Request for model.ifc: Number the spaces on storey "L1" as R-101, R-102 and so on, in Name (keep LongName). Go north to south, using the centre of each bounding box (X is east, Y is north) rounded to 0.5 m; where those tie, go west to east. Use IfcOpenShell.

First a look at what the model holds.

```python
import ifcopenshell
import ifcopenshell.util.element
import ifcopenshell.util.placement

model = ifcopenshell.open("model.ifc")
print(model.schema)
storey = next(s for s in model.by_type("IfcBuildingStorey") if s.Name == "L1")
spaces = [e for e in ifcopenshell.util.element.get_decomposition(storey) if e.is_a("IfcSpace")]
for e in sorted(spaces, key=lambda e: e.id()):
    origin = ifcopenshell.util.placement.get_local_placement(e.ObjectPlacement)[:3, 3]
    print(e.id(), e.Name, e.LongName, origin.round(2) + 0.0, sep=" | ")
```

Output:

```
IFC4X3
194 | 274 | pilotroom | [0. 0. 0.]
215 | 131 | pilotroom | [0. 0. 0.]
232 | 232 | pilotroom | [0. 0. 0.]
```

```python
import ifcopenshell
import ifcopenshell.geom
import ifcopenshell.util.element
import ifcopenshell.util.shape

model = ifcopenshell.open("model.ifc")
settings = ifcopenshell.geom.settings()
settings.set("use-world-coords", True)


def centre(element):
    shape = ifcopenshell.geom.create_shape(settings, element)
    return ifcopenshell.util.shape.get_bbox_centroid(shape.geometry)


storey = next(s for s in model.by_type("IfcBuildingStorey") if s.Name == "L1")
spaces = [e for e in ifcopenshell.util.element.get_decomposition(storey) if e.is_a("IfcSpace")]

# Insertion points can sit at a corner or the storey origin, so sort by the geometry (in metres).
centres = {e: centre(e) for e in spaces}
spaces.sort(key=lambda e: (-round(centres[e][1] / 0.5), centres[e][0]))

for i, e in enumerate(spaces, start=1):
    number = f"R-1{i:02d}"
    e.Name = number
    print(e.id(), number)

model.write("model_v2.ifc")
```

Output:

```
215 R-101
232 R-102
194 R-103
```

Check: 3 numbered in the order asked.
